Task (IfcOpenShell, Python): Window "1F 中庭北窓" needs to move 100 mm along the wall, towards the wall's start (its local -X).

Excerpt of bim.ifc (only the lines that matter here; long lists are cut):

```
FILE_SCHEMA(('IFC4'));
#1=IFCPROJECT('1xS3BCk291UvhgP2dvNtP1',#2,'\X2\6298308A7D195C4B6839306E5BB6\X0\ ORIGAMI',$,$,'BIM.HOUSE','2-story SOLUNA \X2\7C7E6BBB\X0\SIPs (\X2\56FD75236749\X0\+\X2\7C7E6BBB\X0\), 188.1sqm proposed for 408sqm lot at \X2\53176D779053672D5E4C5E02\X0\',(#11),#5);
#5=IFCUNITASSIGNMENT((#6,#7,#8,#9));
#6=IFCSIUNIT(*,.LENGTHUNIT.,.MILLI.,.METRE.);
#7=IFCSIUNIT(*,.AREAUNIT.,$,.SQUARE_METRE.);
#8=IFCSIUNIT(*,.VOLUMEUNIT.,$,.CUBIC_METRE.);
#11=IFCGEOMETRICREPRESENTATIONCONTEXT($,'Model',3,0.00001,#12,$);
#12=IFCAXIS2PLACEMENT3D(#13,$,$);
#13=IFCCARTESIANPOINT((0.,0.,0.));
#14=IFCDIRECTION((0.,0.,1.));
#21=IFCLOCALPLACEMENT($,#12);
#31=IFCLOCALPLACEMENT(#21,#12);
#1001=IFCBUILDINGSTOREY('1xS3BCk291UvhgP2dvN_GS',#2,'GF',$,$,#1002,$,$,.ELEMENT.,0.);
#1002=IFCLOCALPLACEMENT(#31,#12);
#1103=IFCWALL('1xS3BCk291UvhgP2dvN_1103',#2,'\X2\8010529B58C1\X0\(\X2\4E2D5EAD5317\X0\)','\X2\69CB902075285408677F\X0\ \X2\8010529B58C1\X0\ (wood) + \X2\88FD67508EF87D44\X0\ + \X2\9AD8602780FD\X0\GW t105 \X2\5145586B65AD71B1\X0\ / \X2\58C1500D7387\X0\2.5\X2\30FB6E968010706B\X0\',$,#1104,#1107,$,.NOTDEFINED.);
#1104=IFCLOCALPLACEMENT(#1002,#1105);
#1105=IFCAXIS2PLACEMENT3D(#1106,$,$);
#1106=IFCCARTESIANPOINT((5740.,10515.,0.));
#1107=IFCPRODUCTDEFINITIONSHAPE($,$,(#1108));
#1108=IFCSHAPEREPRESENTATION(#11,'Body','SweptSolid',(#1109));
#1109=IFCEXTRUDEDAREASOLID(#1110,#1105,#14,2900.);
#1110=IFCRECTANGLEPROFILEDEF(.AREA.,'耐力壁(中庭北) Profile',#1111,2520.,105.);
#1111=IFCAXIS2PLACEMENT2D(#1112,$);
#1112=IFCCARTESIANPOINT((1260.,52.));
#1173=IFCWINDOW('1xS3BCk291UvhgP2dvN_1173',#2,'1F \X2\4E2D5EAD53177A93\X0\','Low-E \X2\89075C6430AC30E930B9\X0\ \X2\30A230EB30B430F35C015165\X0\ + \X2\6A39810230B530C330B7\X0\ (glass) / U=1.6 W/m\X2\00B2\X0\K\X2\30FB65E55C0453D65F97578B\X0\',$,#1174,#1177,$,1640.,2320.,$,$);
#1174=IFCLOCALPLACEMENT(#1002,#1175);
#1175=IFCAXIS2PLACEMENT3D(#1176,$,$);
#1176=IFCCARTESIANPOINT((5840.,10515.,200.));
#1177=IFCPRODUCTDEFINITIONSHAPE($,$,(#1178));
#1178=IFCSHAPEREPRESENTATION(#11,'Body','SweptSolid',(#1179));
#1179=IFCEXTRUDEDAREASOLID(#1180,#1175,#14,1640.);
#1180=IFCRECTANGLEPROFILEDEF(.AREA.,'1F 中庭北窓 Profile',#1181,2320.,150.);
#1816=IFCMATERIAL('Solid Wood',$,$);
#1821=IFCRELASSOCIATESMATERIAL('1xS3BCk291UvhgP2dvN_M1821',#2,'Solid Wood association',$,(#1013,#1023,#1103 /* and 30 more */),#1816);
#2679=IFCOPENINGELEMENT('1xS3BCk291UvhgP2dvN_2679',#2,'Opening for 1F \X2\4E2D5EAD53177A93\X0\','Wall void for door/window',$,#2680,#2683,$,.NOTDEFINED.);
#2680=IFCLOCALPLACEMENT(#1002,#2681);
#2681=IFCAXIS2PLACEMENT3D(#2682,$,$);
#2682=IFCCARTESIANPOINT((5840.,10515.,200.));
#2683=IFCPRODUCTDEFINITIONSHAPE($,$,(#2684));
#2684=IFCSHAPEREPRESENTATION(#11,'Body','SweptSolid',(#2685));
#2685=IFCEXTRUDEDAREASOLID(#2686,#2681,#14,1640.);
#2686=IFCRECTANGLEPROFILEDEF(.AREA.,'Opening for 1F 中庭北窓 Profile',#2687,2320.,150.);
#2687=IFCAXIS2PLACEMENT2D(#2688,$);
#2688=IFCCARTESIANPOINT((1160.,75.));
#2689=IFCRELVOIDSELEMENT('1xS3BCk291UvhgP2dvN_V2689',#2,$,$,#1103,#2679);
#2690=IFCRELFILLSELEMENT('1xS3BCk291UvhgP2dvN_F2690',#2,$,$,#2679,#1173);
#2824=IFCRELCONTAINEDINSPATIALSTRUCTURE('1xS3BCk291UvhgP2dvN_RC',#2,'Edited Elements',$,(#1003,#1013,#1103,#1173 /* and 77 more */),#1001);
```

```python
import ifcopenshell
import ifcopenshell.api.geometry
import ifcopenshell.util.placement
import ifcopenshell.util.unit

model = ifcopenshell.open("bim.ifc")
unit_scale = ifcopenshell.util.unit.calculate_unit_scale(model)

window = model.by_guid("1xS3BCk291UvhgP2dvN_1173")
opening = window.FillsVoids[0].RelatingOpeningElement
wall = opening.VoidsElements[0].RelatingBuildingElement

wall_matrix = ifcopenshell.util.placement.get_local_placement(wall.ObjectPlacement)
shift = wall_matrix[:3, 0] * -0.1 / unit_scale
before = ifcopenshell.util.placement.get_local_placement(window.ObjectPlacement)[:3, 3].copy()

# The window is not placed relative to its opening, so move both.
for product in (opening, window):
    matrix = ifcopenshell.util.placement.get_local_placement(product.ObjectPlacement)
    matrix[:3, 3] += shift
    ifcopenshell.api.geometry.edit_object_placement(model, product=product, matrix=matrix, is_si=False)

after = ifcopenshell.util.placement.get_local_placement(window.ObjectPlacement)[:3, 3]
print("window moved by", (after - before).round(3) + 0.0)

model.write("bim_rev.ifc")
```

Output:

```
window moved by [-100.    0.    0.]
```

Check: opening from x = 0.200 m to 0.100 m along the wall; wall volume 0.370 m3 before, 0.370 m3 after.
